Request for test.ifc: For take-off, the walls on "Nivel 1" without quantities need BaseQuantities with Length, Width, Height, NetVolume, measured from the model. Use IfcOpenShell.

First a look at what the model holds.

```python
import ifcopenshell
import ifcopenshell.util.element
import ifcopenshell.util.unit

model = ifcopenshell.open("test.ifc")
print(model.schema)
for unit_type in ("LENGTHUNIT", "AREAUNIT", "VOLUMEUNIT"):
    print(unit_type, ifcopenshell.util.unit.calculate_unit_scale(model, unit_type))
storey = next(s for s in model.by_type("IfcBuildingStorey") if s.Name == "Nivel 1")
walls = [e for e in ifcopenshell.util.element.get_decomposition(storey) if e.is_a("IfcWall")]
for e in sorted(walls, key=lambda e: e.id()):
    print(e.id(), e.is_a(), e.Name, list(ifcopenshell.util.element.get_psets(e, qtos_only=True)), sep=" | ")
```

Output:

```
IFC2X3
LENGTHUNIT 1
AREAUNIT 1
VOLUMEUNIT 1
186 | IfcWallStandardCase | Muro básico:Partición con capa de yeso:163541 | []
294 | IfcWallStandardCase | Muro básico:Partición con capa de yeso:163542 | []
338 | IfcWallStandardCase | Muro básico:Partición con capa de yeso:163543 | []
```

```python
import ifcopenshell
import ifcopenshell.api.pset
import ifcopenshell.geom
import ifcopenshell.util.element
import ifcopenshell.util.shape
import ifcopenshell.util.unit

model = ifcopenshell.open("test.ifc")
unit_scale = ifcopenshell.util.unit.calculate_unit_scale(model)
volume_scale = ifcopenshell.util.unit.calculate_unit_scale(model, "VOLUMEUNIT")
settings = ifcopenshell.geom.settings()

storey = next(s for s in model.by_type("IfcBuildingStorey") if s.Name == "Nivel 1")
walls = [e for e in ifcopenshell.util.element.get_decomposition(storey) if e.is_a("IfcWall")]

for e in sorted(walls, key=lambda e: e.id()):
    if ifcopenshell.util.element.get_psets(e, qtos_only=True, should_inherit=False):
        continue
    # Geometry comes back in metres, in the element's own axes.
    shape = ifcopenshell.geom.create_shape(settings, e)
    values = {
        "Length": ifcopenshell.util.shape.get_x(shape.geometry) / unit_scale,
        "Width": ifcopenshell.util.shape.get_y(shape.geometry) / unit_scale,
        "Height": ifcopenshell.util.shape.get_z(shape.geometry) / unit_scale,
        "NetVolume": ifcopenshell.util.shape.get_volume(shape.geometry) / volume_scale,
    }
    qto = ifcopenshell.api.pset.add_qto(model, product=e, name="BaseQuantities")
    ifcopenshell.api.pset.edit_qto(model, qto=qto, properties=values)
    print(e.id(), {k: round(v, 3) for k, v in values.items()})

model.write("test_edited.ifc")
```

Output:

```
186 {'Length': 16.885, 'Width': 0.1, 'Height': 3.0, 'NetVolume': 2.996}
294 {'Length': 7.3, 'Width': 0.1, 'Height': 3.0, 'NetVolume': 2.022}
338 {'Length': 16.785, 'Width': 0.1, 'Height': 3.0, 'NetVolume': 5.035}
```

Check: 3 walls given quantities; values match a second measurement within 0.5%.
